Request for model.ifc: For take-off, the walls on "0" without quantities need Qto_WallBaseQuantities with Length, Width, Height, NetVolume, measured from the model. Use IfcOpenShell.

First a look at what the model holds.

```python
import ifcopenshell
import ifcopenshell.util.element
import ifcopenshell.util.unit

model = ifcopenshell.open("model.ifc")
print(model.schema)
for unit_type in ("LENGTHUNIT", "AREAUNIT", "VOLUMEUNIT"):
    print(unit_type, ifcopenshell.util.unit.calculate_unit_scale(model, unit_type))
storey = next(s for s in model.by_type("IfcBuildingStorey") if s.Name == "0")
walls = [e for e in ifcopenshell.util.element.get_decomposition(storey) if e.is_a("IfcWall")]
for e in sorted(walls, key=lambda e: e.id()):
    print(e.id(), e.is_a(), e.Name, list(ifcopenshell.util.element.get_psets(e, qtos_only=True)), sep=" | ")
```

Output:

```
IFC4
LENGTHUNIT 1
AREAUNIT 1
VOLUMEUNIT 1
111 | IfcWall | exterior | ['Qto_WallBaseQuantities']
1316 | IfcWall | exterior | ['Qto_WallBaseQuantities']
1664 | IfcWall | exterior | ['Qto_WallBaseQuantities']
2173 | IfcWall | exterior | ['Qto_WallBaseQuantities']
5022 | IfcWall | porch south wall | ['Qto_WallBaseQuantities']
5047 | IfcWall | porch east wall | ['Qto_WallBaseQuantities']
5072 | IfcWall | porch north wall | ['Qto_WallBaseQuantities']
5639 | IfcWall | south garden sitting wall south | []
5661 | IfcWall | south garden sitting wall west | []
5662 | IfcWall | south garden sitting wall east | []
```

```python
import ifcopenshell
import ifcopenshell.api.pset
import ifcopenshell.geom
import ifcopenshell.util.element
import ifcopenshell.util.shape
import ifcopenshell.util.unit

model = ifcopenshell.open("model.ifc")
unit_scale = ifcopenshell.util.unit.calculate_unit_scale(model)
volume_scale = ifcopenshell.util.unit.calculate_unit_scale(model, "VOLUMEUNIT")
settings = ifcopenshell.geom.settings()

storey = next(s for s in model.by_type("IfcBuildingStorey") if s.Name == "0")
walls = [e for e in ifcopenshell.util.element.get_decomposition(storey) if e.is_a("IfcWall")]

for e in sorted(walls, key=lambda e: e.id()):
    if ifcopenshell.util.element.get_psets(e, qtos_only=True, should_inherit=False):
        continue
    # Geometry comes back in metres, in the element's own axes.
    shape = ifcopenshell.geom.create_shape(settings, e)
    values = {
        "Length": ifcopenshell.util.shape.get_x(shape.geometry) / unit_scale,
        "Width": ifcopenshell.util.shape.get_y(shape.geometry) / unit_scale,
        "Height": ifcopenshell.util.shape.get_z(shape.geometry) / unit_scale,
        "NetVolume": ifcopenshell.util.shape.get_volume(shape.geometry) / volume_scale,
    }
    qto = ifcopenshell.api.pset.add_qto(model, product=e, name="Qto_WallBaseQuantities")
    ifcopenshell.api.pset.edit_qto(model, qto=qto, properties=values)
    print(e.id(), {k: round(v, 3) for k, v in values.items()})

model.write("model_edited.ifc")
```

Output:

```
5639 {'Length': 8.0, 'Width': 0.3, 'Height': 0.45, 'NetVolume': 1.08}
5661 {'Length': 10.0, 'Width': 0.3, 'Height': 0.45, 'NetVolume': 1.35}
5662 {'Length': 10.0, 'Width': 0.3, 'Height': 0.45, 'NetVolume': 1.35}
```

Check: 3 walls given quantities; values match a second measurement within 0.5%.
